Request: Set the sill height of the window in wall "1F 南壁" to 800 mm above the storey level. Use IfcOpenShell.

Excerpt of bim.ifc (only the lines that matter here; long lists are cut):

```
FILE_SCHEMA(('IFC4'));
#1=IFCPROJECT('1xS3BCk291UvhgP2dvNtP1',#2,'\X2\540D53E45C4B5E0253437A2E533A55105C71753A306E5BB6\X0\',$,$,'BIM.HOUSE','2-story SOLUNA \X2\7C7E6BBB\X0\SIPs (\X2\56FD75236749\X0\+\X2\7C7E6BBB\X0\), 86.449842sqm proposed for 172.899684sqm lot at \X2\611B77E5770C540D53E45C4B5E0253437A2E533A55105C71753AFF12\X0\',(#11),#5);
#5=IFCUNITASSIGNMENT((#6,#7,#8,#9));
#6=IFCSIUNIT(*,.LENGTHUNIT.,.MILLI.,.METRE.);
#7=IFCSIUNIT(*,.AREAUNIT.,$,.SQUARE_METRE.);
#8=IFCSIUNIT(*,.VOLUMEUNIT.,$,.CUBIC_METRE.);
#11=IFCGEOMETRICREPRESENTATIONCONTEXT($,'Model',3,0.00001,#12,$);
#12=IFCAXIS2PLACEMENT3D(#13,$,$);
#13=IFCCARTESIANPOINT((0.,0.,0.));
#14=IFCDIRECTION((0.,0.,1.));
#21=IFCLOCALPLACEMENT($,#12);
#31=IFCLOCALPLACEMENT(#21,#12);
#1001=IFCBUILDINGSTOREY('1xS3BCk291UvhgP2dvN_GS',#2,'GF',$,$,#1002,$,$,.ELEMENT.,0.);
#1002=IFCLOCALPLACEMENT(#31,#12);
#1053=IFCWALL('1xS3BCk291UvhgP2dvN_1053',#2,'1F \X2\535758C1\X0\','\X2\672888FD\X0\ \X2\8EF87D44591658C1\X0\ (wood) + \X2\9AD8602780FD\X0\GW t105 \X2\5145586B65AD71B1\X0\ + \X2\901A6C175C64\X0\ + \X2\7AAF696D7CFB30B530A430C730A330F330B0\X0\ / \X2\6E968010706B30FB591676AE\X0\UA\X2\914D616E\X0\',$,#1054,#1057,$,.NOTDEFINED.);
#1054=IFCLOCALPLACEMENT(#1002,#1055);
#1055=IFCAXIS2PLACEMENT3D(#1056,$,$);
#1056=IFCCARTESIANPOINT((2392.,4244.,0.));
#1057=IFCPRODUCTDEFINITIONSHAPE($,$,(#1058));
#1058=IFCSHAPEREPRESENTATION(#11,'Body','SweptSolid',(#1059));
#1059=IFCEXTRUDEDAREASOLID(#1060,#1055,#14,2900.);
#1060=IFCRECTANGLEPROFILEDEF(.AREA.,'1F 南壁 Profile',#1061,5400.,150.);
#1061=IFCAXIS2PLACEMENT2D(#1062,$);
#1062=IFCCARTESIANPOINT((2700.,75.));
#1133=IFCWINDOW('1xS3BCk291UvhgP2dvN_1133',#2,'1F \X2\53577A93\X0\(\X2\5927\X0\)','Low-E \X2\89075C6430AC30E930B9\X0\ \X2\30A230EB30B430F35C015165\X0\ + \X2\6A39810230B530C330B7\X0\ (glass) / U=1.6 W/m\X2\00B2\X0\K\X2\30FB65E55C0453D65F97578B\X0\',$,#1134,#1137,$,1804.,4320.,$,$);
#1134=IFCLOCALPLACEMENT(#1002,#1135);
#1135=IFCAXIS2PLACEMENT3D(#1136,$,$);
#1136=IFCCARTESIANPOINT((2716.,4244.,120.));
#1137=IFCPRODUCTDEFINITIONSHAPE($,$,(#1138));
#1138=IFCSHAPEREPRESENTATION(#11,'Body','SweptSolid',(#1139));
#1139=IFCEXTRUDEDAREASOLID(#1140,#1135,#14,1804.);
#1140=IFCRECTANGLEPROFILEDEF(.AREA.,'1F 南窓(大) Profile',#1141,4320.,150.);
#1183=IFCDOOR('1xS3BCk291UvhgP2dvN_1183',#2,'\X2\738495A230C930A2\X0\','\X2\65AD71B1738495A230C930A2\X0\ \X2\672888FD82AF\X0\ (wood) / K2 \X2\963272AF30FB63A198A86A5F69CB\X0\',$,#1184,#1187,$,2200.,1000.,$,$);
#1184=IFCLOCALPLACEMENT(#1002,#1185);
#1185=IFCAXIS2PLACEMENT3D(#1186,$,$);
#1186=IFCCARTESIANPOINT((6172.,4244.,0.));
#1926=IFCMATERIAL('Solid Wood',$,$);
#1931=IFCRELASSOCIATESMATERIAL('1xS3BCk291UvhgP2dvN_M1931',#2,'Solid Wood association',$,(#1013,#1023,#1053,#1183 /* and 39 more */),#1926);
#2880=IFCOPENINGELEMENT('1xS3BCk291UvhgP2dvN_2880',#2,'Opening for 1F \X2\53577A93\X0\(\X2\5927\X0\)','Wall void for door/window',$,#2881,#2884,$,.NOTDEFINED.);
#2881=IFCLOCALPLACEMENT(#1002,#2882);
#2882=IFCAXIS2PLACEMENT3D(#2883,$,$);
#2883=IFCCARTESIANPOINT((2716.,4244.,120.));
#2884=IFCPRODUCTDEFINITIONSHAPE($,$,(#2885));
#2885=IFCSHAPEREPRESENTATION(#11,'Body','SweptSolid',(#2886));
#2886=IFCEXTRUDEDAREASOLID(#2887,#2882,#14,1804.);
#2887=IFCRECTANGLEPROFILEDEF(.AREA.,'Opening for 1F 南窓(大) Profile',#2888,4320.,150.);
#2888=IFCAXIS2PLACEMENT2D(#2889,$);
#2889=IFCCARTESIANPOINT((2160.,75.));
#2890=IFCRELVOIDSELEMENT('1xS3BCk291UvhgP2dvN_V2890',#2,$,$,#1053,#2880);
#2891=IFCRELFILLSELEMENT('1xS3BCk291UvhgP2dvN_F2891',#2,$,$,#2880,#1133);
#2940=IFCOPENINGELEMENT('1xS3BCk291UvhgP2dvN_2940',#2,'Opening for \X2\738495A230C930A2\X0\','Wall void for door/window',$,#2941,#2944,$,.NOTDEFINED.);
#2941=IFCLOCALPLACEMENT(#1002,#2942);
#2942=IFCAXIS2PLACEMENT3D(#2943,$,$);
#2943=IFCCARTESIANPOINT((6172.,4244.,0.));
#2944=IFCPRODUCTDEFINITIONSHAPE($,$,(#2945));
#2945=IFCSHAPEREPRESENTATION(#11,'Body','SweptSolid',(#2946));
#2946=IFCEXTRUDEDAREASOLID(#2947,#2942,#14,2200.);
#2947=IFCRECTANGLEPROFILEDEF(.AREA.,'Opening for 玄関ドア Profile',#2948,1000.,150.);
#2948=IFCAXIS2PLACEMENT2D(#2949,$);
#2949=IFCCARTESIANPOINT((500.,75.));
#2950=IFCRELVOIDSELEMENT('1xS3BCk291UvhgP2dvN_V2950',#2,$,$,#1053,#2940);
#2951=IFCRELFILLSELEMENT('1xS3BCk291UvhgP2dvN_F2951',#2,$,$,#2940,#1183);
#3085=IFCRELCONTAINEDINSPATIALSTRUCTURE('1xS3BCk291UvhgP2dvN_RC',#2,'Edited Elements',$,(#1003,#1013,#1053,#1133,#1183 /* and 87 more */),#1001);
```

```python
import numpy as np
import ifcopenshell
import ifcopenshell.api.geometry
import ifcopenshell.geom
import ifcopenshell.util.element
import ifcopenshell.util.placement
import ifcopenshell.util.shape
import ifcopenshell.util.unit

model = ifcopenshell.open("bim.ifc")
unit_scale = ifcopenshell.util.unit.calculate_unit_scale(model)

window = model.by_guid("1xS3BCk291UvhgP2dvN_1133")
opening = window.FillsVoids[0].RelatingOpeningElement
storey = ifcopenshell.util.element.get_container(window, ifc_class="IfcBuildingStorey")
level = ifcopenshell.util.placement.get_local_placement(storey.ObjectPlacement)[2, 3]

# The opening's origin need not be at the sill, so measure its lowest point.
shape = ifcopenshell.geom.create_shape(ifcopenshell.geom.settings(), opening)
bottom = ifcopenshell.util.shape.get_shape_bottom_elevation(shape, shape.geometry) / unit_scale
dz = level + 0.8 / unit_scale - bottom

shift = np.array([0.0, 0.0, dz])
# The window is not placed relative to its opening, so move both.
for product in (opening, window):
    matrix = ifcopenshell.util.placement.get_local_placement(product.ObjectPlacement)
    matrix[:3, 3] += shift
    ifcopenshell.api.geometry.edit_object_placement(model, product=product, matrix=matrix, is_si=False)

print(f"moved by {dz * unit_scale:+.3f} m")

model.write("bim_v2.ifc")
```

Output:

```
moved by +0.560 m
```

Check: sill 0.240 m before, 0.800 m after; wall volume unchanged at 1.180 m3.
